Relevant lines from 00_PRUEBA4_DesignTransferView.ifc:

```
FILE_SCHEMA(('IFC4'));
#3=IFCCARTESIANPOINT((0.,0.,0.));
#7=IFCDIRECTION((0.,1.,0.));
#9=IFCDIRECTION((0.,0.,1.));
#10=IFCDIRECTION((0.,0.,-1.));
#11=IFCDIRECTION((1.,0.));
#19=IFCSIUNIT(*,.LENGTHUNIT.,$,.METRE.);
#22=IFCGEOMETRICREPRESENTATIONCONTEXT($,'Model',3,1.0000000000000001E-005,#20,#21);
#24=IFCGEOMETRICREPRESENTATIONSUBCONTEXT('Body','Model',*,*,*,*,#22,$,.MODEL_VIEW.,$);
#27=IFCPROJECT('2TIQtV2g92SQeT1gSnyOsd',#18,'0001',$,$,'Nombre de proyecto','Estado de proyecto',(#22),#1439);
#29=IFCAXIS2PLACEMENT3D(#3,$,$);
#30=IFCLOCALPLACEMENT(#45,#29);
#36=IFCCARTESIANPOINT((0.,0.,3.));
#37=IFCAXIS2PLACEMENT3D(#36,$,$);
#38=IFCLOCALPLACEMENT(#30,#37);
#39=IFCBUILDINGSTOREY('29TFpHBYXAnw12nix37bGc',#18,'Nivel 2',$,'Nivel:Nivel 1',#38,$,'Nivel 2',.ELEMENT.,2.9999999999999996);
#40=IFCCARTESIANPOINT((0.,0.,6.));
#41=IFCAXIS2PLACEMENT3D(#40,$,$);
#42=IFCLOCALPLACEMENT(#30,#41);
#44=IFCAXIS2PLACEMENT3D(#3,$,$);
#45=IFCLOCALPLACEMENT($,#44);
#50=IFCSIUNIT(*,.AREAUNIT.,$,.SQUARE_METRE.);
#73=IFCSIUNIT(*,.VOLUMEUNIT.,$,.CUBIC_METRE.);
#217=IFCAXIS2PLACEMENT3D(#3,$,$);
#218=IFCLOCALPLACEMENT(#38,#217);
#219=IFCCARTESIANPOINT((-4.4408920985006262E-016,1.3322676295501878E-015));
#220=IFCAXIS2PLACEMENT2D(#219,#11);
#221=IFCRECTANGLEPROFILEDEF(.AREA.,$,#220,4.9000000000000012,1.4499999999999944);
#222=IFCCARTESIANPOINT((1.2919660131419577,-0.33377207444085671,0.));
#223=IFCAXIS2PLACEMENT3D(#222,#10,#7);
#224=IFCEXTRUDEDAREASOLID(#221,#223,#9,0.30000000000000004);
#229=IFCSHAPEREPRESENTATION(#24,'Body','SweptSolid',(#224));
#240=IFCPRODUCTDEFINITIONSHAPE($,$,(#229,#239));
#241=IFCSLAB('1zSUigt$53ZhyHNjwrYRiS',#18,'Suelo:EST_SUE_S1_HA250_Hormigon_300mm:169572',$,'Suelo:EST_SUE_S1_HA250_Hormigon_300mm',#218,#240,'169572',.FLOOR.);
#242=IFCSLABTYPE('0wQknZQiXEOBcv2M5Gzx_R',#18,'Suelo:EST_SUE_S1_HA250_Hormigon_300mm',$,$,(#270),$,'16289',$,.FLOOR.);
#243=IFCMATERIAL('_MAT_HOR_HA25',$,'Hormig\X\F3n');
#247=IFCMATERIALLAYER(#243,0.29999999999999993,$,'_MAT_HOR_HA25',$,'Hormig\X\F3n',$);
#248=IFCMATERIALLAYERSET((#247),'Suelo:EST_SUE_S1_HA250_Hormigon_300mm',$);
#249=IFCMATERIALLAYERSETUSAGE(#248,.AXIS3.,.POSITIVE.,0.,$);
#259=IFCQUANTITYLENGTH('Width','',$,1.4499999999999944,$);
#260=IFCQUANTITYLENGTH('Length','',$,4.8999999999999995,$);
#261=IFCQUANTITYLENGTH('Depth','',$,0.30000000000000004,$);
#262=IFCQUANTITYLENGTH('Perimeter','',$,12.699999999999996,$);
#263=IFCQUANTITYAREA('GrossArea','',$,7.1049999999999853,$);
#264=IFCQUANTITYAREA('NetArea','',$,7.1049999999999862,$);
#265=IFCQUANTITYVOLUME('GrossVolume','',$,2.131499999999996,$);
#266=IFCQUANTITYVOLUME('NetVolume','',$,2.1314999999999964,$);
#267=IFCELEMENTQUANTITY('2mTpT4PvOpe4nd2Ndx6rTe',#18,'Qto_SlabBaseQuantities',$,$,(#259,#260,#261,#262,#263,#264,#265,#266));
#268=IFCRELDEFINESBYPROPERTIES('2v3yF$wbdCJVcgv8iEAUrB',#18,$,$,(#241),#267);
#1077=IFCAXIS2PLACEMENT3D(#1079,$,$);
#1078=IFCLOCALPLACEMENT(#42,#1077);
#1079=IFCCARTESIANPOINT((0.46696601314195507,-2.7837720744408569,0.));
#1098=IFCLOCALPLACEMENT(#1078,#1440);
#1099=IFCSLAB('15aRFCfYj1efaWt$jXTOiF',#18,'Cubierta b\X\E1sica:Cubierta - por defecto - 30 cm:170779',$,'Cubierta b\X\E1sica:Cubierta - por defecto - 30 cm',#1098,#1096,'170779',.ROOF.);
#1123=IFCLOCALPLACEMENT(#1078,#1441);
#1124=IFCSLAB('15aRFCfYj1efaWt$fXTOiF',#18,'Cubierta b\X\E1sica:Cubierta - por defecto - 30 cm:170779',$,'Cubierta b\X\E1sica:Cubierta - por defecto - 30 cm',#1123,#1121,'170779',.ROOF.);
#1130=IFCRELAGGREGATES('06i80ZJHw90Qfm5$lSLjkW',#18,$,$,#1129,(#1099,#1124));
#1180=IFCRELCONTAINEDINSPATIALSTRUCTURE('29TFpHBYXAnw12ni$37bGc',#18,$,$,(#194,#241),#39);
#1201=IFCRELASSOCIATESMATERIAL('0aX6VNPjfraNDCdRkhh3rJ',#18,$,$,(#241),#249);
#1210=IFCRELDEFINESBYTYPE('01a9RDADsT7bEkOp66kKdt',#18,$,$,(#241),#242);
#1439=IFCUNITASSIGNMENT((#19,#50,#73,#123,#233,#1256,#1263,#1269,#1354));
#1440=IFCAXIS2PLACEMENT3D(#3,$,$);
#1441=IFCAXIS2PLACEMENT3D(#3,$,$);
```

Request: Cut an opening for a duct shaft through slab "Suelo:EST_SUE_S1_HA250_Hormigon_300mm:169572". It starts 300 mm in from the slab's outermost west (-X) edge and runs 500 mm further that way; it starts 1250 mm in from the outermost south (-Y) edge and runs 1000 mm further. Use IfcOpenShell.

```python
import numpy as np
import ifcopenshell
import ifcopenshell.api.feature
import ifcopenshell.api.geometry
import ifcopenshell.api.pset
import ifcopenshell.api.root
import ifcopenshell.geom
import ifcopenshell.util.element
import ifcopenshell.util.placement
import ifcopenshell.util.representation
import ifcopenshell.util.shape
import ifcopenshell.util.unit

model = ifcopenshell.open("00_PRUEBA4_DesignTransferView.ifc")
unit_scale = ifcopenshell.util.unit.calculate_unit_scale(model)
area_scale = ifcopenshell.util.unit.calculate_unit_scale(model, "AREAUNIT")
volume_scale = ifcopenshell.util.unit.calculate_unit_scale(model, "VOLUMEUNIT")
settings = ifcopenshell.geom.settings()


def volume(element):
    """Net volume in cubic metres, openings subtracted."""
    shape = ifcopenshell.geom.create_shape(settings, element)
    return ifcopenshell.util.shape.get_volume(shape.geometry)


slab = model.by_guid("1zSUigt$53ZhyHNjwrYRiS")
before = volume(slab)

# Extent in the slab's own axes, in metres. The edges named are its -X and -Y sides.
slab_shape = ifcopenshell.geom.create_shape(settings, slab)
vertices = ifcopenshell.util.shape.get_vertices(slab_shape.geometry)
x_min, y_min, bottom = vertices.min(axis=0)
top = vertices[:, 2].max()

opening = ifcopenshell.api.root.create_entity(model, ifc_class="IfcOpeningElement", name="Duct shaft opening", predefined_type="OPENING")
context = ifcopenshell.util.representation.get_context(model, "Model", "Body", "MODEL_VIEW")
width, depth = 0.5, 1
outline = [(0.0, 0.0), (width, 0.0), (width, depth), (0.0, depth), (0.0, 0.0)]
# Overshoot both faces by 50 mm so the cut is clean.
shape = ifcopenshell.api.geometry.add_slab_representation(
    model, context=context, depth=top - bottom + 0.1, polyline=outline
)
ifcopenshell.api.geometry.assign_representation(model, product=opening, representation=shape)

matrix = ifcopenshell.util.placement.get_local_placement(slab.ObjectPlacement)
matrix[:, 3] = matrix @ np.append(np.array([x_min + 0.3, y_min + 1.25, bottom - 0.05]) / unit_scale, 1.0)
ifcopenshell.api.geometry.edit_object_placement(model, product=opening, matrix=matrix, is_si=False)
ifcopenshell.api.feature.add_feature(model, feature=opening, element=slab)

after = volume(slab)

# Update the slab's stored quantities.
qto = model.by_id(ifcopenshell.util.element.get_pset(slab, "Qto_SlabBaseQuantities", should_inherit=False)["id"])
ifcopenshell.api.pset.edit_qto(model, qto=qto, properties={
    "NetArea": after / (top - bottom) / area_scale,
    "NetVolume": after / volume_scale,
})

print(f"slab volume {before:.3f} -> {after:.3f} m3")

model.write("00_PRUEBA4_DesignTransferView_v2.ifc")
```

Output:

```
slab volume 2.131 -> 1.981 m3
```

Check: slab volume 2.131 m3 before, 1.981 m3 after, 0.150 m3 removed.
